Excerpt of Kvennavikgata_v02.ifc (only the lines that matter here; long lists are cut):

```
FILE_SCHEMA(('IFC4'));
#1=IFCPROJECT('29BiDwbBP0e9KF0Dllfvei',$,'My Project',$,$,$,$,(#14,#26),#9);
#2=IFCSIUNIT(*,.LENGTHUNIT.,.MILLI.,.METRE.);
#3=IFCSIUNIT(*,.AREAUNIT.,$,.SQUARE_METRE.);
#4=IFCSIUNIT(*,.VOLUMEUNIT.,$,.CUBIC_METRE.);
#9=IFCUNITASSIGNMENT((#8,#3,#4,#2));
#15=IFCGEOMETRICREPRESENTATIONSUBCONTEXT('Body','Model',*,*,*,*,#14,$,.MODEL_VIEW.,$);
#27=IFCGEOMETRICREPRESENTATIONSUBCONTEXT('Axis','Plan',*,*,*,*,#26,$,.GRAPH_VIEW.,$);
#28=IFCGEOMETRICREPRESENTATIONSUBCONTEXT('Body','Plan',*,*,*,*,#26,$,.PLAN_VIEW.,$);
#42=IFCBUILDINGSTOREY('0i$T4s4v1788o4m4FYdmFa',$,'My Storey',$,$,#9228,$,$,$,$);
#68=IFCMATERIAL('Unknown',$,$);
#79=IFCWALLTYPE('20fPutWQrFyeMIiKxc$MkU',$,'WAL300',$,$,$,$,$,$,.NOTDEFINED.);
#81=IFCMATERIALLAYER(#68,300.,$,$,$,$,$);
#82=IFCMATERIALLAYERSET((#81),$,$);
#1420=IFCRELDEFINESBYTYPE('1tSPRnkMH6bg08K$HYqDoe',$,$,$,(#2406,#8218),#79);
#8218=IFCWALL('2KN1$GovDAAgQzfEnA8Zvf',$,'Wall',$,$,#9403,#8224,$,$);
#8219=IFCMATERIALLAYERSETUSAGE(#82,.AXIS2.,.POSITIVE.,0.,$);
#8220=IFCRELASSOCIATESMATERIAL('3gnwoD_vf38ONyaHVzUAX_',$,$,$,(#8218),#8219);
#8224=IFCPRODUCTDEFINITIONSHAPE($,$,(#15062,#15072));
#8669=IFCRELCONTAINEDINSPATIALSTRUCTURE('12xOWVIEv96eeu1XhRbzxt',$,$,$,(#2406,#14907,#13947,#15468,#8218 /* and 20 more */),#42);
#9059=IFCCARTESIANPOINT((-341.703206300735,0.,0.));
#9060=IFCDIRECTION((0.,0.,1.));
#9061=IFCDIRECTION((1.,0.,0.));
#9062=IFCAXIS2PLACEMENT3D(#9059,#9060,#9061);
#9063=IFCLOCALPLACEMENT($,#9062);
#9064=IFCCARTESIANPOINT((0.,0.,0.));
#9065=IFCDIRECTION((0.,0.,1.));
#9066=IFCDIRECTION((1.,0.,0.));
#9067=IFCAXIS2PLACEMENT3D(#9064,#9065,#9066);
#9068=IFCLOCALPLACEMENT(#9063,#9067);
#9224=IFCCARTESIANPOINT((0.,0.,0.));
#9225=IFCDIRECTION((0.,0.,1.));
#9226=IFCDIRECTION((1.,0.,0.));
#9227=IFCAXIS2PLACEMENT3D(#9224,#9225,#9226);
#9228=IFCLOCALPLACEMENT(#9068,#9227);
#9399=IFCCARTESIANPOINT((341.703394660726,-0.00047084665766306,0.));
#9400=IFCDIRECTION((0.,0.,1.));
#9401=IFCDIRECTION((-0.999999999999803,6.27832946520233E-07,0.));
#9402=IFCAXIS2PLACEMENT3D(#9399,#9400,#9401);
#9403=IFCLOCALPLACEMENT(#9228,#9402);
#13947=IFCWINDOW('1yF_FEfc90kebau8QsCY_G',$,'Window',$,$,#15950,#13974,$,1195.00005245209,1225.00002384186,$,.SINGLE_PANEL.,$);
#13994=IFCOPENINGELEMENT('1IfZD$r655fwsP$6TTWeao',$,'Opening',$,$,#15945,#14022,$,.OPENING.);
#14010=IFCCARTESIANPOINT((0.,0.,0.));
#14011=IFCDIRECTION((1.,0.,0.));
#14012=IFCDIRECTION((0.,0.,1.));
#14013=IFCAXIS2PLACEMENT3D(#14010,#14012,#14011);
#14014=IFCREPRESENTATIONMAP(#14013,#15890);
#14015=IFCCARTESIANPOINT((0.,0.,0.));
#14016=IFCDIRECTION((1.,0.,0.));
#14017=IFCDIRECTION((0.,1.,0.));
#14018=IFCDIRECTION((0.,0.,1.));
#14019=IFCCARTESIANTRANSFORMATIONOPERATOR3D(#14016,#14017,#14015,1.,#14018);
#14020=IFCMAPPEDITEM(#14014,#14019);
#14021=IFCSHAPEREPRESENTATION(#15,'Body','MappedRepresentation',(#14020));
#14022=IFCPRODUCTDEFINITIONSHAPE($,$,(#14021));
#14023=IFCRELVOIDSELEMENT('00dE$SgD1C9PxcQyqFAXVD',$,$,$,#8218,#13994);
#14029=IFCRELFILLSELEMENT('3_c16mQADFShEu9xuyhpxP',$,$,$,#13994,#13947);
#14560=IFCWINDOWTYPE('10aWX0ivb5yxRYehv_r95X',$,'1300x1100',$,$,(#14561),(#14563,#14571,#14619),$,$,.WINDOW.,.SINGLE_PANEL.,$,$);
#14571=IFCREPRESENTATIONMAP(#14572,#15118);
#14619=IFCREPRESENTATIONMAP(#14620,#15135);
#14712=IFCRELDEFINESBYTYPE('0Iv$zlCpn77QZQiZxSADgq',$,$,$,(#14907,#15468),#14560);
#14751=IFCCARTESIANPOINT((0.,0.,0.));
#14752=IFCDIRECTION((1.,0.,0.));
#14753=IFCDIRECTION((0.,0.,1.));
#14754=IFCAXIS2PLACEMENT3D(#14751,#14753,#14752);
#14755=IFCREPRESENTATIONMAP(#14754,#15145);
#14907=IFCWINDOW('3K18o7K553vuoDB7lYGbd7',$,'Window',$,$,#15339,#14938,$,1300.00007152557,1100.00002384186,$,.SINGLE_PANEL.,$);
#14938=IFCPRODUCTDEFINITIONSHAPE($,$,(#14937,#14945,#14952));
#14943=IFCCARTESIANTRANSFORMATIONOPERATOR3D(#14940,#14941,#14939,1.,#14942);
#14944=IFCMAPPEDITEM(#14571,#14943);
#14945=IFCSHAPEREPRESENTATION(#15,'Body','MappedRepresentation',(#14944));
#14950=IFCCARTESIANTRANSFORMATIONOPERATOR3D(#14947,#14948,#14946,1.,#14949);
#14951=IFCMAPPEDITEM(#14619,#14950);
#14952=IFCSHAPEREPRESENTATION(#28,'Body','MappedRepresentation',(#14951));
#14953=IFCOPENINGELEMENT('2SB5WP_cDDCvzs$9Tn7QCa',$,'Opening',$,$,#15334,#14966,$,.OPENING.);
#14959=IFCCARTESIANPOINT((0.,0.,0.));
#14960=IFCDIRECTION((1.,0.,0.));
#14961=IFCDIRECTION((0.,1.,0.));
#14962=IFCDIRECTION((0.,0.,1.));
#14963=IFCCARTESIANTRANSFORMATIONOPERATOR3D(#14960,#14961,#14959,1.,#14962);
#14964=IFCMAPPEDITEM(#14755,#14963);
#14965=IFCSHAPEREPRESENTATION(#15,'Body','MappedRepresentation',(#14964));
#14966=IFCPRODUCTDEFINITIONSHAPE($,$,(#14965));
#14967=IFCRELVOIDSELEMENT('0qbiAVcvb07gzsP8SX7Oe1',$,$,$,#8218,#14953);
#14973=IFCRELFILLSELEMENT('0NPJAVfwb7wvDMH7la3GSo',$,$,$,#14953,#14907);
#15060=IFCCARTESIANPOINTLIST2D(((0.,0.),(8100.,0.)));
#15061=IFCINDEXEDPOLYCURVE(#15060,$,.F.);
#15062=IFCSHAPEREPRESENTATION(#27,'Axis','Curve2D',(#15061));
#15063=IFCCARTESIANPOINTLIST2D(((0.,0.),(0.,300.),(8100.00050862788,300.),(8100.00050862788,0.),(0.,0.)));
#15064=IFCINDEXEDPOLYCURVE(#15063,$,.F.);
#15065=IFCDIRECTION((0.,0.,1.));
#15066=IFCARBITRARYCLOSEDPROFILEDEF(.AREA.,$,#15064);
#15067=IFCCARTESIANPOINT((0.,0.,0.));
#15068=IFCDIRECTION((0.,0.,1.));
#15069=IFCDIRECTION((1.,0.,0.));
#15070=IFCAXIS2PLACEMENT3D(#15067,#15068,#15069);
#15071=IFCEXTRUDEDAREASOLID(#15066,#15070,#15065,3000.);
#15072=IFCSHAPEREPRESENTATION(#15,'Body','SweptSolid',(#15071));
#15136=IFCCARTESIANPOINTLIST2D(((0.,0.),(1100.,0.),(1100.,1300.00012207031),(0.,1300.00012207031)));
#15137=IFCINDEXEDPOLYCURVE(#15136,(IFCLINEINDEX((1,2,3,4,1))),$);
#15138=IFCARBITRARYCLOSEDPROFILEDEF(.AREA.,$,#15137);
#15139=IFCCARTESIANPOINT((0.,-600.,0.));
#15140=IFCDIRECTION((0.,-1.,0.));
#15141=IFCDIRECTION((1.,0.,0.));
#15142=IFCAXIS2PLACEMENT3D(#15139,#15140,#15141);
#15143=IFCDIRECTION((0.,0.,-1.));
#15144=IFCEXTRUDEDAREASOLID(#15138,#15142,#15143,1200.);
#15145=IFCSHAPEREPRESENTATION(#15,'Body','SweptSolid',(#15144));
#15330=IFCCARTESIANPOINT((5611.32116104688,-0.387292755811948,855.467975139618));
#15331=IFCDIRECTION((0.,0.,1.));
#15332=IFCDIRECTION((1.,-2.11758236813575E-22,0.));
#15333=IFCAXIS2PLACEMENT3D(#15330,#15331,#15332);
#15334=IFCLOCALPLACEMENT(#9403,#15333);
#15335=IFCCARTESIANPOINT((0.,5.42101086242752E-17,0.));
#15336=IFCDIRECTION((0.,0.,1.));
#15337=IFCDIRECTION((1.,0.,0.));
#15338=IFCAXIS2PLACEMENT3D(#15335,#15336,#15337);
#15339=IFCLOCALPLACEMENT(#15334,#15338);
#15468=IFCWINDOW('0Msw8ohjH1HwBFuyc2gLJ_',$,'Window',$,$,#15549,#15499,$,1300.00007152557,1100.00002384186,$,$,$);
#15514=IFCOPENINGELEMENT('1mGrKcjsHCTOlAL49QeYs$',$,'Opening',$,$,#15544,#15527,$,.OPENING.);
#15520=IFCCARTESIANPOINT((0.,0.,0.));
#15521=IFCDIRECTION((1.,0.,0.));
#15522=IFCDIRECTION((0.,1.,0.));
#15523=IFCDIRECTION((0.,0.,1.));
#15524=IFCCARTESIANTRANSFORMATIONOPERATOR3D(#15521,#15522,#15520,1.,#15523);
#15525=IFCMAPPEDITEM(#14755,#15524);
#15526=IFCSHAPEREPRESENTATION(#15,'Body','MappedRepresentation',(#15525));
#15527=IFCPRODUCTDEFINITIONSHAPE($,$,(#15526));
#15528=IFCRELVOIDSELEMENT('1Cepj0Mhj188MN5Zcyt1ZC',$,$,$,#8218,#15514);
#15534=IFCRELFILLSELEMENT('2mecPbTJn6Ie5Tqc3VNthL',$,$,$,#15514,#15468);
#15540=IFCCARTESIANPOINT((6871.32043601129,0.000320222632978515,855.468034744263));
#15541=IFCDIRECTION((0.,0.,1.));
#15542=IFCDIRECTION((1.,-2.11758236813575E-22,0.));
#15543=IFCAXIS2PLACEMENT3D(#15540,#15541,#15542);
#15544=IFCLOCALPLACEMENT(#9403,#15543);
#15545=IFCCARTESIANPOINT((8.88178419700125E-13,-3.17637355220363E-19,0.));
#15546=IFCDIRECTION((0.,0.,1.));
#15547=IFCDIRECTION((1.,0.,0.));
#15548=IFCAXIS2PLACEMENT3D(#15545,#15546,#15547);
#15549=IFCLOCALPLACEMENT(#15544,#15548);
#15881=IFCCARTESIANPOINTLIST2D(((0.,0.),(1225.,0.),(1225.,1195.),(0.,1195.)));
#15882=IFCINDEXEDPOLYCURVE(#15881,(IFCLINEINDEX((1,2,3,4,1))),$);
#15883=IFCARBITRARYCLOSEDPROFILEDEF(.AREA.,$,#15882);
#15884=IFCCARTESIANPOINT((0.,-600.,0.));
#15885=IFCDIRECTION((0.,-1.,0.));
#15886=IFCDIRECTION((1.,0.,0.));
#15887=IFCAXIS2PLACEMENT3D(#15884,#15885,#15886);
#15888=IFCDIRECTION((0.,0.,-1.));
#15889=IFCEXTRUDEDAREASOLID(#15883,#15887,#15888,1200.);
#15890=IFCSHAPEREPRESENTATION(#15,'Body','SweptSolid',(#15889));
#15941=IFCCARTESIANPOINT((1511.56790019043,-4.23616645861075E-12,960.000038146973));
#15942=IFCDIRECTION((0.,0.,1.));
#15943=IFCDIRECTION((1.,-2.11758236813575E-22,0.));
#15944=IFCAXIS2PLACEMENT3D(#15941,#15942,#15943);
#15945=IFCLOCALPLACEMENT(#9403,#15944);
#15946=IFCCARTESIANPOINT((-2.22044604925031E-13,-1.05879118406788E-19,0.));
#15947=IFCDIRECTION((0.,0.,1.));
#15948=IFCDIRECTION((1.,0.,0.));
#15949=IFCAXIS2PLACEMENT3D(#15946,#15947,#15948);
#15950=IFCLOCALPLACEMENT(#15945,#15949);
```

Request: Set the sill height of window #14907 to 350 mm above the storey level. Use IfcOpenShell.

```python
import numpy as np
import ifcopenshell
import ifcopenshell.api.geometry
import ifcopenshell.geom
import ifcopenshell.util.element
import ifcopenshell.util.placement
import ifcopenshell.util.shape
import ifcopenshell.util.unit

model = ifcopenshell.open("Kvennavikgata_v02.ifc")
unit_scale = ifcopenshell.util.unit.calculate_unit_scale(model)

window = model.by_guid("3K18o7K553vuoDB7lYGbd7")
opening = window.FillsVoids[0].RelatingOpeningElement
storey = ifcopenshell.util.element.get_container(window, ifc_class="IfcBuildingStorey")
level = ifcopenshell.util.placement.get_local_placement(storey.ObjectPlacement)[2, 3]

# The opening's origin need not be at the sill, so measure its lowest point.
shape = ifcopenshell.geom.create_shape(ifcopenshell.geom.settings(), opening)
bottom = ifcopenshell.util.shape.get_shape_bottom_elevation(shape, shape.geometry) / unit_scale
dz = level + 0.35 / unit_scale - bottom

shift = np.array([0.0, 0.0, dz])
# The window is placed relative to its opening, so it follows when the opening moves.
matrix = ifcopenshell.util.placement.get_local_placement(opening.ObjectPlacement)
matrix[:3, 3] += shift
ifcopenshell.api.geometry.edit_object_placement(
    model, product=opening, matrix=matrix, is_si=False, should_transform_children=True
)

print(f"moved by {dz * unit_scale:+.3f} m")

model.write("Kvennavikgata_v02_rev.ifc")
```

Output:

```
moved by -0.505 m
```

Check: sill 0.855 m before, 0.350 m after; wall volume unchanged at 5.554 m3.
